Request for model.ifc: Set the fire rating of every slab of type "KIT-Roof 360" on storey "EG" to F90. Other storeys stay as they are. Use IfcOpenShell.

First a look at what the model holds.

```python
import ifcopenshell
import ifcopenshell.util.element

model = ifcopenshell.open("model.ifc")
print(model.schema)
storey = next(s for s in model.by_type("IfcBuildingStorey") if s.Name == "EG")
slabs = [e for e in ifcopenshell.util.element.get_decomposition(storey) if e.is_a("IfcSlab")]
seen = {}
for e in slabs:
    element_type = ifcopenshell.util.element.get_type(e)
    key = (element_type.Name if element_type != e and element_type else None, ifcopenshell.util.element.get_pset(e, "Pset_SlabCommon", "FireRating"))
    seen[key] = seen.get(key, 0) + 1
for (name, value), count in sorted(seen.items(), key=str):
    print(count, "x", name, "|", value)
```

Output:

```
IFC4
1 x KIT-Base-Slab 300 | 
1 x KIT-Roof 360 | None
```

```python
import ifcopenshell
import ifcopenshell.api.pset
import ifcopenshell.util.element

model = ifcopenshell.open("model.ifc")

storey = next(s for s in model.by_type("IfcBuildingStorey") if s.Name == "EG")
slabs = [e for e in ifcopenshell.util.element.get_decomposition(storey) if e.is_a("IfcSlab")]

count = 0
for e in slabs:
    element_type = ifcopenshell.util.element.get_type(e)
    if element_type in (None, e) or element_type.Name != "KIT-Roof 360":
        continue
    # add_pset returns the element's existing set when there is one.
    pset = ifcopenshell.api.pset.add_pset(model, product=e, name="Pset_SlabCommon")
    ifcopenshell.api.pset.edit_pset(model, pset=pset, properties={"FireRating": "F90"})
    count += 1

print(count, "slabs updated")

model.write("model_rev.ifc")
```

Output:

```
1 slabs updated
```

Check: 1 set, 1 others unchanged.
